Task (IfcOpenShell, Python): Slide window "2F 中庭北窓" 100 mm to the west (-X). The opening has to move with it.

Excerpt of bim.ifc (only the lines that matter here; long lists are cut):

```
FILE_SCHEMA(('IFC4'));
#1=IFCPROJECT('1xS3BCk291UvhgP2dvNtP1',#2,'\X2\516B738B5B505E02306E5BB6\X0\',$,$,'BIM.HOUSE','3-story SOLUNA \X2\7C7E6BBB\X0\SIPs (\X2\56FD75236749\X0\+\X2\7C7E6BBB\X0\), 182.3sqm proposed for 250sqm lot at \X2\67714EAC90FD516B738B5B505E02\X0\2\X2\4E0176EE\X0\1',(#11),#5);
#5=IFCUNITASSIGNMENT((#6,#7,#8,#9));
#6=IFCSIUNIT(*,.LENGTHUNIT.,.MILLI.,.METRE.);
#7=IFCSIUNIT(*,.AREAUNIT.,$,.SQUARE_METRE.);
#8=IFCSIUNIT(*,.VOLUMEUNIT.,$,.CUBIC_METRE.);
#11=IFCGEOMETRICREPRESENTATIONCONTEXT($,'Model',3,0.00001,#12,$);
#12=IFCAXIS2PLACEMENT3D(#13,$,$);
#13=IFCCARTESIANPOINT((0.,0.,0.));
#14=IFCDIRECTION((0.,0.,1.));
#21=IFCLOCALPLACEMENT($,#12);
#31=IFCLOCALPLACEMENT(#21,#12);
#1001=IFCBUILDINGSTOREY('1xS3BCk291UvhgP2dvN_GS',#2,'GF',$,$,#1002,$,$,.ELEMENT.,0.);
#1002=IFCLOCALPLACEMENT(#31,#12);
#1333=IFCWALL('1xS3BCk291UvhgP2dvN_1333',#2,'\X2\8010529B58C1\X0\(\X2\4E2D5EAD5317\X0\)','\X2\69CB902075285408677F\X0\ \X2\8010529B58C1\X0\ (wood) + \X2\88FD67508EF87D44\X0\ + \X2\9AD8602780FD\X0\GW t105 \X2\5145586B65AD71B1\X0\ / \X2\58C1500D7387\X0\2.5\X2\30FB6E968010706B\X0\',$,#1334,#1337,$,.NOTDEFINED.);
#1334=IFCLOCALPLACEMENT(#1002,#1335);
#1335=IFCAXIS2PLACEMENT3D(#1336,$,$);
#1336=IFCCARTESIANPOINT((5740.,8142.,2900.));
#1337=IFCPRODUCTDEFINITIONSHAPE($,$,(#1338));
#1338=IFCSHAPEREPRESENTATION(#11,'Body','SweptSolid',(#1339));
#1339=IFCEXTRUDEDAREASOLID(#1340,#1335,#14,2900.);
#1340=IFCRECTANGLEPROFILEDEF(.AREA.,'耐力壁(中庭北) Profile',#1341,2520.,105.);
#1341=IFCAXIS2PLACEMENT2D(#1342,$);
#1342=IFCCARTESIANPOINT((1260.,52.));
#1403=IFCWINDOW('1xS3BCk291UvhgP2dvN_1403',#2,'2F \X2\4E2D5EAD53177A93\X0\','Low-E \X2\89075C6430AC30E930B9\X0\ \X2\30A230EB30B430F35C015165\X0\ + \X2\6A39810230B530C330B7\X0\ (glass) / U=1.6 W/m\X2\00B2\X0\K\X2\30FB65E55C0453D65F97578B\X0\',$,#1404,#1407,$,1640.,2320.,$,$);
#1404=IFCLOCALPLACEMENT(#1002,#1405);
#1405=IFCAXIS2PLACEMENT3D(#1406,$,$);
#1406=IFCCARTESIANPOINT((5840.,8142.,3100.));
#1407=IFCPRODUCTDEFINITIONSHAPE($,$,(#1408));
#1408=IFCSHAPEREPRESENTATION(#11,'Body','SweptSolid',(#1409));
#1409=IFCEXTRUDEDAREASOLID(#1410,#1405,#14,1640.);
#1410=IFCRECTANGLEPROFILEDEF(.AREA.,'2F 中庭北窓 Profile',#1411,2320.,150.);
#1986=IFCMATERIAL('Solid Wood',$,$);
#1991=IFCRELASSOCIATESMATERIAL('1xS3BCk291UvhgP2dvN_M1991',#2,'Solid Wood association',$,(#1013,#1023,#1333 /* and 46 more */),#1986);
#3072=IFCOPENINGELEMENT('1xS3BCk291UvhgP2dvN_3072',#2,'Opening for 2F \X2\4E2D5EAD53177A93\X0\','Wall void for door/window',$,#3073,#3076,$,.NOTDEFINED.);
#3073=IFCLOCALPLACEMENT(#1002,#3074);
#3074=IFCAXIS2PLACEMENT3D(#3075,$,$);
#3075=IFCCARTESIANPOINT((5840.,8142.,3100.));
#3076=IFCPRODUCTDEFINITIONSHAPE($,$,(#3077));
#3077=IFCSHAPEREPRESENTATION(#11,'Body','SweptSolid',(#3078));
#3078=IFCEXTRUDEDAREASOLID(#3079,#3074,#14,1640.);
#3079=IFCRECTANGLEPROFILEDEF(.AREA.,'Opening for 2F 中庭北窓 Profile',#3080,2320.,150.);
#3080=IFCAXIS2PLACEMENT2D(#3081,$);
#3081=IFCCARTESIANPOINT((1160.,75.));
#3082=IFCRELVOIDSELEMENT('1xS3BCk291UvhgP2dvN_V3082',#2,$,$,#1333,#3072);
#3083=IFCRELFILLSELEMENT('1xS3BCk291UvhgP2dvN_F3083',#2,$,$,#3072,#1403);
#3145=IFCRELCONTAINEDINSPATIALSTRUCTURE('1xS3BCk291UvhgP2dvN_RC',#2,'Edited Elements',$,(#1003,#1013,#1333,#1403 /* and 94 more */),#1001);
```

```python
import ifcopenshell
import ifcopenshell.api.geometry
import ifcopenshell.util.placement
import ifcopenshell.util.unit

model = ifcopenshell.open("bim.ifc")
unit_scale = ifcopenshell.util.unit.calculate_unit_scale(model)

window = model.by_id(1403)
opening = window.FillsVoids[0].RelatingOpeningElement
wall = opening.VoidsElements[0].RelatingBuildingElement

wall_matrix = ifcopenshell.util.placement.get_local_placement(wall.ObjectPlacement)
shift = wall_matrix[:3, 0] * -0.1 / unit_scale
before = ifcopenshell.util.placement.get_local_placement(window.ObjectPlacement)[:3, 3].copy()

# The window is not placed relative to its opening, so move both.
for product in (opening, window):
    matrix = ifcopenshell.util.placement.get_local_placement(product.ObjectPlacement)
    matrix[:3, 3] += shift
    ifcopenshell.api.geometry.edit_object_placement(model, product=product, matrix=matrix, is_si=False)

after = ifcopenshell.util.placement.get_local_placement(window.ObjectPlacement)[:3, 3]
print("window moved by", (after - before).round(3) + 0.0)

model.write("bim_rev.ifc")
```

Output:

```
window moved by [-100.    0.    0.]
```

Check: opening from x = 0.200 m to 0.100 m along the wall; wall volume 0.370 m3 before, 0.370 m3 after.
